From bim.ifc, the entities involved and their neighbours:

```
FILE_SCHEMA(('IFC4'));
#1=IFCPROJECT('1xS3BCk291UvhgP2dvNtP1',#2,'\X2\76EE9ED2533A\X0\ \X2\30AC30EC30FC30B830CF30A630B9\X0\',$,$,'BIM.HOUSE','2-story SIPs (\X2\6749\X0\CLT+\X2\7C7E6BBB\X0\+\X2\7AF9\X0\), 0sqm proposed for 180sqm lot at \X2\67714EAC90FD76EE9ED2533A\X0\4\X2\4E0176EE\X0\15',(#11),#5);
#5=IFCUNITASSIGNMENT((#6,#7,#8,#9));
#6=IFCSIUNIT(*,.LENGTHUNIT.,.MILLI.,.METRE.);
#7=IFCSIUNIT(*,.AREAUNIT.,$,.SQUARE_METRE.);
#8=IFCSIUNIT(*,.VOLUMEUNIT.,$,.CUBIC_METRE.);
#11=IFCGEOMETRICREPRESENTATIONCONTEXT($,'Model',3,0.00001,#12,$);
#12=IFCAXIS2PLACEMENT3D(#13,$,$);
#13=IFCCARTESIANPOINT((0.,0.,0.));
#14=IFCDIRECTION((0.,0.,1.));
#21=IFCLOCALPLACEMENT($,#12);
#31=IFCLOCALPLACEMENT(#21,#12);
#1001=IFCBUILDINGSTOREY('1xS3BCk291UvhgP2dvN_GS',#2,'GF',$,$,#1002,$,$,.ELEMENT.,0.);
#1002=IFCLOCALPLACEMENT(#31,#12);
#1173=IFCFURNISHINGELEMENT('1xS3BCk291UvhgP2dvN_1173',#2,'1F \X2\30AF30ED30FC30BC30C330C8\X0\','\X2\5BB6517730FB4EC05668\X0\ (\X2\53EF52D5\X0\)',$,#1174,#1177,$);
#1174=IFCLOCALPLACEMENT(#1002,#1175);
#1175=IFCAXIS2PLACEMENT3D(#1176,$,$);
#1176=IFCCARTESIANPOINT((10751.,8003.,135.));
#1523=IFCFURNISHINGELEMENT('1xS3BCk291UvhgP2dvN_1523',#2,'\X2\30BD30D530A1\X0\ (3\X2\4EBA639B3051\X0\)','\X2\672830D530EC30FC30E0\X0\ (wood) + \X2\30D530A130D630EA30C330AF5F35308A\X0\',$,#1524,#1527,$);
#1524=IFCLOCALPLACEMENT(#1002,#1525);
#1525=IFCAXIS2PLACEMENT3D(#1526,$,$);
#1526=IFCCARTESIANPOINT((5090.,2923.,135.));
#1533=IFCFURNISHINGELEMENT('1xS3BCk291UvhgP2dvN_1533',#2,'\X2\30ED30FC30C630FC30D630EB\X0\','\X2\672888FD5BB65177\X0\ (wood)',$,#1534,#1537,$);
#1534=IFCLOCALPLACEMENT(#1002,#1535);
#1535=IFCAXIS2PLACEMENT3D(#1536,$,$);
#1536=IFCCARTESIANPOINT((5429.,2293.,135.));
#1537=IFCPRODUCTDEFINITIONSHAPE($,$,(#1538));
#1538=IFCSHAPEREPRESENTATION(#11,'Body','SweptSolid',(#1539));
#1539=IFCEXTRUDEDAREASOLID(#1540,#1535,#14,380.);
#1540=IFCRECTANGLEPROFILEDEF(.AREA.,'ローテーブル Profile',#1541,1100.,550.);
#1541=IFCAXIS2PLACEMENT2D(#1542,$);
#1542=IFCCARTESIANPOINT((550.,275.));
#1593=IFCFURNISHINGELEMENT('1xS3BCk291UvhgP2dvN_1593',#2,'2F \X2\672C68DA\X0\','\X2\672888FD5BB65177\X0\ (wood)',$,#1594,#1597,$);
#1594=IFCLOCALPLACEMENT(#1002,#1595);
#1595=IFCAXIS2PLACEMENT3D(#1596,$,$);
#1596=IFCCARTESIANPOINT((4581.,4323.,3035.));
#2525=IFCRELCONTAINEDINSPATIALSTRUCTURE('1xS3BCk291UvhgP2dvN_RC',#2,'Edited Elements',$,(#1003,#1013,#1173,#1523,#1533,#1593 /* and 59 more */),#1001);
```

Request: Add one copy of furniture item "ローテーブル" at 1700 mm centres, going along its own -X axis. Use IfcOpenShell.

```python
import ifcopenshell
import ifcopenshell.api.geometry
import ifcopenshell.api.root
import ifcopenshell.util.element
import ifcopenshell.util.placement

model = ifcopenshell.open("bim.ifc")


def reuse_history(source, copy):
    """copy_class also copies each property set's owner history, people and application; keep the originals."""
    for rel in copy.IsDefinedBy:
        if rel.is_a("IfcRelDefinesByProperties") and (history := rel.RelatingPropertyDefinition.OwnerHistory):
            rel.RelatingPropertyDefinition.OwnerHistory = source.OwnerHistory
            ifcopenshell.util.element.remove_deep2(model, history)


source = model.by_id(1533)
base = ifcopenshell.util.placement.get_local_placement(source.ObjectPlacement)
step = -base[:3, 0] * 1700.0

for i in range(1, 2):
    copy = ifcopenshell.api.root.copy_class(model, product=source)
    copy.Representation = ifcopenshell.util.element.copy_deep(
        model, source.Representation, exclude=["IfcGeometricRepresentationContext", "IfcRepresentationMap"]
    )
    reuse_history(source, copy)
    matrix = base.copy()
    matrix[:3, 3] += i * step
    print("added at", matrix[:3, 3].round(3) + 0.0)
    ifcopenshell.api.geometry.edit_object_placement(model, product=copy, matrix=matrix, is_si=False)

model.write("bim_v2.ifc")
```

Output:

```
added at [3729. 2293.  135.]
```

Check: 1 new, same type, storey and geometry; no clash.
